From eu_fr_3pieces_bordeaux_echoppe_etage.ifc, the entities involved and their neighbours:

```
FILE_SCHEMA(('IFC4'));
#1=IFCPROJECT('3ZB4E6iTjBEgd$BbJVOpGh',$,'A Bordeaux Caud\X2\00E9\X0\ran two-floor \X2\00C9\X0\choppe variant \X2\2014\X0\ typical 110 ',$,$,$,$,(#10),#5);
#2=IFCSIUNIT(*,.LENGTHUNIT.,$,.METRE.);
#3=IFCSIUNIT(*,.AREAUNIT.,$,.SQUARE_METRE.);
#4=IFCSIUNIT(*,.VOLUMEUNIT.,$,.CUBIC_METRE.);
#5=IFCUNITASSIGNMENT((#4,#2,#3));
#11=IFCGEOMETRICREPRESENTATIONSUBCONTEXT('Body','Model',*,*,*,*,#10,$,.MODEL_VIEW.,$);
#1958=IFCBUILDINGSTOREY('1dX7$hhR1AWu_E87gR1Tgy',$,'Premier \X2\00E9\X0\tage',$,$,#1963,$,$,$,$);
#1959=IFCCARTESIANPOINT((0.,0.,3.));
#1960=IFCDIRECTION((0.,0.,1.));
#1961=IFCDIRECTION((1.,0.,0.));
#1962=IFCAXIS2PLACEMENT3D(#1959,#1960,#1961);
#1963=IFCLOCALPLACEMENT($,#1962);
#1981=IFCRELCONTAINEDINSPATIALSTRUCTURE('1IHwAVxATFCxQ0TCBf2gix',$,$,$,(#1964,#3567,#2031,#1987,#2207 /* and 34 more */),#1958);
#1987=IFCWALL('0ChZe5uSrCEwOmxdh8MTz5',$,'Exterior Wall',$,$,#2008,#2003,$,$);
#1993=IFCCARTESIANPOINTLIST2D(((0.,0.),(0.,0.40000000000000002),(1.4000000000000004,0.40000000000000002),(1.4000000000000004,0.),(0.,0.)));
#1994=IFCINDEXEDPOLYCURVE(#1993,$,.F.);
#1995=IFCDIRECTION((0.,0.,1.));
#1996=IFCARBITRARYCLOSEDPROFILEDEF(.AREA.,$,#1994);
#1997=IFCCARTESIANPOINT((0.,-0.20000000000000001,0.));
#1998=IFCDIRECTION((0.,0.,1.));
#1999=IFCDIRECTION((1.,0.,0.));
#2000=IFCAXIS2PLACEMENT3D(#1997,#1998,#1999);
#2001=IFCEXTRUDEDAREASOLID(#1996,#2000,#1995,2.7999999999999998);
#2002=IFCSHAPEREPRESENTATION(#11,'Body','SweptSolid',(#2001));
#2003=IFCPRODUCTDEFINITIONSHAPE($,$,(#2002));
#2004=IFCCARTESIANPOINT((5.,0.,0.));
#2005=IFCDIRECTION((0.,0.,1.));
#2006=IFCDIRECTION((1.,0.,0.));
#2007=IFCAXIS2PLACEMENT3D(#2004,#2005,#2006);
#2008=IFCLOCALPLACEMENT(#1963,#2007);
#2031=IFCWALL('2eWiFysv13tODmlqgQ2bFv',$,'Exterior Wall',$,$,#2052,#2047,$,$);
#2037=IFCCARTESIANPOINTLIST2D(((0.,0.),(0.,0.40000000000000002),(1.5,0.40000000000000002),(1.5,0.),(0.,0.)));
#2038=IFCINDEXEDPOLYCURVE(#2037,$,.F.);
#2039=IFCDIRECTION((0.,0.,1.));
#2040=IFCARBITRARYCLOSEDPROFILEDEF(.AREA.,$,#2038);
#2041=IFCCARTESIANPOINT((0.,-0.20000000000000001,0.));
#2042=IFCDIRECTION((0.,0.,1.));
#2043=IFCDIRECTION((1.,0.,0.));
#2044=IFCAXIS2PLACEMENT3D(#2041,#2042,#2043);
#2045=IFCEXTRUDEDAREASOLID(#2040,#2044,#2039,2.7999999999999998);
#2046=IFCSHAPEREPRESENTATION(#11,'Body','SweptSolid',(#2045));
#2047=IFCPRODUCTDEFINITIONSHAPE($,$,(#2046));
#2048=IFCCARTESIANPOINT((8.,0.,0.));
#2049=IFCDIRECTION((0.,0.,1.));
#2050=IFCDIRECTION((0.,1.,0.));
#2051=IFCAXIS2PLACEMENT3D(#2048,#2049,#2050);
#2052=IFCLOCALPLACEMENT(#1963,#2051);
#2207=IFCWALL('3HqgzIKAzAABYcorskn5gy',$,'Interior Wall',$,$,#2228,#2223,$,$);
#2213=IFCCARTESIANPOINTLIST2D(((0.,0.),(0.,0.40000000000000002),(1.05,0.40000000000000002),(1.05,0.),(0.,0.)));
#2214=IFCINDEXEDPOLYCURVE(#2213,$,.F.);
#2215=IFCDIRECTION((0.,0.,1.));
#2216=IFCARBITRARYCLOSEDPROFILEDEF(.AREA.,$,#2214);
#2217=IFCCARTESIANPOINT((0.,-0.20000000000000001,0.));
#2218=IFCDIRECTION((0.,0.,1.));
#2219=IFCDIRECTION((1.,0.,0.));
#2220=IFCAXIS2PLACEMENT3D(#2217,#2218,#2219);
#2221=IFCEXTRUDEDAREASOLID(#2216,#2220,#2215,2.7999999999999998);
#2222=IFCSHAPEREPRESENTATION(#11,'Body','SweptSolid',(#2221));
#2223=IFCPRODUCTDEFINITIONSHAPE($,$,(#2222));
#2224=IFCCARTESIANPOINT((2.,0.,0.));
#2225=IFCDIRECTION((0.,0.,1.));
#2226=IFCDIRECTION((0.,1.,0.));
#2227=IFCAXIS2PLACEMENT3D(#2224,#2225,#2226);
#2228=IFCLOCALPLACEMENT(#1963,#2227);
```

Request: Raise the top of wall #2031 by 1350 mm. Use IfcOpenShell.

```python
import ifcopenshell
import ifcopenshell.geom
import ifcopenshell.util.representation
import ifcopenshell.util.shape
import ifcopenshell.util.unit

model = ifcopenshell.open("eu_fr_3pieces_bordeaux_echoppe_etage.ifc")
unit_scale = ifcopenshell.util.unit.calculate_unit_scale(model)
settings = ifcopenshell.geom.settings()


def volume(element):
    """Net volume in cubic metres, openings subtracted."""
    shape = ifcopenshell.geom.create_shape(settings, element)
    return ifcopenshell.util.shape.get_volume(shape.geometry)


wall = model.by_guid("2eWiFysv13tODmlqgQ2bFv")
before = volume(wall)

body = ifcopenshell.util.representation.get_representation(wall, "Model", "Body")
solid = body.Items[0]
old_height = solid.Depth
solid.Depth += 1.35 / unit_scale
after = volume(wall)

print(f"height {old_height:g} -> {solid.Depth:g}, volume {before:.3f} -> {after:.3f} m3")

model.write("eu_fr_3pieces_bordeaux_echoppe_etage_edited.ifc")
```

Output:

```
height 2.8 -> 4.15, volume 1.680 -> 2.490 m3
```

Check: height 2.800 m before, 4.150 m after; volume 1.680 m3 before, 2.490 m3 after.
